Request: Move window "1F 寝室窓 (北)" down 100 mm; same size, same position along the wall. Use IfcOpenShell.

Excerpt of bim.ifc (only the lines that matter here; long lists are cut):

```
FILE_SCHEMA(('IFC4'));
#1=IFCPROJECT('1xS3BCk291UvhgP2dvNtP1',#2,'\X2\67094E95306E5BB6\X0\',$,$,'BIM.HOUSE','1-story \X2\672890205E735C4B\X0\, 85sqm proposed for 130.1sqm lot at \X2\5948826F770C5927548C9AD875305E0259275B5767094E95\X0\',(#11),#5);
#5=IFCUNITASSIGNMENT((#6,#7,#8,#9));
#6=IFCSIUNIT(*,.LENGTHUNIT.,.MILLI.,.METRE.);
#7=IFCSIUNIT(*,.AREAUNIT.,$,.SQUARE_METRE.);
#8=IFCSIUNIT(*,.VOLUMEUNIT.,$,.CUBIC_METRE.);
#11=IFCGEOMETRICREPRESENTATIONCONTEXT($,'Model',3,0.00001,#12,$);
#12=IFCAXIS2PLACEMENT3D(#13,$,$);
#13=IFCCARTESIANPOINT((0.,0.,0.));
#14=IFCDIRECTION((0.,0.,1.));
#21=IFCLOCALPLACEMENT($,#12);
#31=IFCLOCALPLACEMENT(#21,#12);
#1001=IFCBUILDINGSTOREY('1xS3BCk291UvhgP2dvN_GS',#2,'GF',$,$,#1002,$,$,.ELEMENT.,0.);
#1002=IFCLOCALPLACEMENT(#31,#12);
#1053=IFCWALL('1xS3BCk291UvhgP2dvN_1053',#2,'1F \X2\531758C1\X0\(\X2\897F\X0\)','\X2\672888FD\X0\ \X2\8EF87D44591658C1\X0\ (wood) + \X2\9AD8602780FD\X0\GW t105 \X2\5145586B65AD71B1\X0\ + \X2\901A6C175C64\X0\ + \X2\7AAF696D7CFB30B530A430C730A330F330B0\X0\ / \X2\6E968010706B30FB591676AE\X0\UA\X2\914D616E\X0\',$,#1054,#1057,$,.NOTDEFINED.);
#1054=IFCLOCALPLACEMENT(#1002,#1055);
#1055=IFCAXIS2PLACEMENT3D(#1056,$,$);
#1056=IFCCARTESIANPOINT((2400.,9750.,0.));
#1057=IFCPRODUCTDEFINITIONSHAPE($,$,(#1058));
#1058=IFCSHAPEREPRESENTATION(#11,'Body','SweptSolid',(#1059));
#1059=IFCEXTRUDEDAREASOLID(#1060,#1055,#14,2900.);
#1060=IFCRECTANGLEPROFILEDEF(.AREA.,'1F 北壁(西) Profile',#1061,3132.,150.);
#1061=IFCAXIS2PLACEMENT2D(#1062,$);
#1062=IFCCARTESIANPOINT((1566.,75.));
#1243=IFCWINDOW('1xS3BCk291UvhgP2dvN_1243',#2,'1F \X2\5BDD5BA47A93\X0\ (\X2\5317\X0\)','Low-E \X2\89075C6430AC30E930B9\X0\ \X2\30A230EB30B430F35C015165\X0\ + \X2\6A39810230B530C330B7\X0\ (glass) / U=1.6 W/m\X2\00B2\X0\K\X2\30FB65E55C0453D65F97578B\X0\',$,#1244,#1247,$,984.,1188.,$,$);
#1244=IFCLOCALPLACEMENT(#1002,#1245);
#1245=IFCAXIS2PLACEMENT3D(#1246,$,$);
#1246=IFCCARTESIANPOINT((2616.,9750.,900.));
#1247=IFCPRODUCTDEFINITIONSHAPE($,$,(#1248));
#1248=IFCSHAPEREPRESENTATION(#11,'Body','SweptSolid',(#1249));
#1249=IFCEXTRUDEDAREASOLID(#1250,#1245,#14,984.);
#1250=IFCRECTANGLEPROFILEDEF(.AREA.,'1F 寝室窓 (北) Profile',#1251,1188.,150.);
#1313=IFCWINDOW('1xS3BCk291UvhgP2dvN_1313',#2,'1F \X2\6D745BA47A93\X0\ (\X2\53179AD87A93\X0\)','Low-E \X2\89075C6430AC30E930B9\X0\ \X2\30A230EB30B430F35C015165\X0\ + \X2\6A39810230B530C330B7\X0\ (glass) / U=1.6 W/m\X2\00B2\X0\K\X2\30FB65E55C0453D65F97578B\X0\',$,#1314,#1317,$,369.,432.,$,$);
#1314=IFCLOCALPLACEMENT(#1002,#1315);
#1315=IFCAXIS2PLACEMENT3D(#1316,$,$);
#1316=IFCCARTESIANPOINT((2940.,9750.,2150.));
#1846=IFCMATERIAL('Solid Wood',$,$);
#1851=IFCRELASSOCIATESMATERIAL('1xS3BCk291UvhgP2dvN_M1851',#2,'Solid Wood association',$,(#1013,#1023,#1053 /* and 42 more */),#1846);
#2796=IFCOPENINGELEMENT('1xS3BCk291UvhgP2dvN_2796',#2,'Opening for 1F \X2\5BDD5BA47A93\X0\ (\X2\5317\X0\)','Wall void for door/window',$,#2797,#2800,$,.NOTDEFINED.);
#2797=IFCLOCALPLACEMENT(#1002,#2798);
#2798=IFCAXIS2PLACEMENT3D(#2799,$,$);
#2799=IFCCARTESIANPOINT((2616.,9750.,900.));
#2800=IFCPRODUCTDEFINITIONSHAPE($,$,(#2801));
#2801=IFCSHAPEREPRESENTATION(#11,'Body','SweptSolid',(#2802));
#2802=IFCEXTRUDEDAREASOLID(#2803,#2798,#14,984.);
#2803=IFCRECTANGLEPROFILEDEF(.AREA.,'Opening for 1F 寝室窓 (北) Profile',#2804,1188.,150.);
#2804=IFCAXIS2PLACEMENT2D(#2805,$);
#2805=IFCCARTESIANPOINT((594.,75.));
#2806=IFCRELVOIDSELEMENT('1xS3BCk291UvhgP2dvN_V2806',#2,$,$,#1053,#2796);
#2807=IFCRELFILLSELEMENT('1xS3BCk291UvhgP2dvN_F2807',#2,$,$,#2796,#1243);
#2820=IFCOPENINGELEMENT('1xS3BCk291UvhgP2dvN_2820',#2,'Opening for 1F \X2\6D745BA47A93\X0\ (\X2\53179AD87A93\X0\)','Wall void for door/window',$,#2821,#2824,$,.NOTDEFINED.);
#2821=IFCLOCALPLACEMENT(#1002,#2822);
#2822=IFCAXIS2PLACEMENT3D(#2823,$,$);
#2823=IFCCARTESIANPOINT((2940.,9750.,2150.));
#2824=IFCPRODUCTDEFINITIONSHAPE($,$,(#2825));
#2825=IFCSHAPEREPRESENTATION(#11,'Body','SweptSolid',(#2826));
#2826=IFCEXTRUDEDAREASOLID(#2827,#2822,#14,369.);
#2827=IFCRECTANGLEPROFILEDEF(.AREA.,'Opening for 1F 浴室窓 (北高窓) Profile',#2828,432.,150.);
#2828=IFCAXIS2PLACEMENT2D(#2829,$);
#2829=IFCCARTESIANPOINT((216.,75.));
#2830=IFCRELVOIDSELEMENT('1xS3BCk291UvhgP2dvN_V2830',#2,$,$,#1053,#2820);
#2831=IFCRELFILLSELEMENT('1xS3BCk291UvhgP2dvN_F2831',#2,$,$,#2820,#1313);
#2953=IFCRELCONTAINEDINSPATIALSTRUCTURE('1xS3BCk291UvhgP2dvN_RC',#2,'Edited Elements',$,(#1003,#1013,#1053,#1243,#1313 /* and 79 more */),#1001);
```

```python
import numpy as np
import ifcopenshell
import ifcopenshell.api.geometry
import ifcopenshell.util.placement
import ifcopenshell.util.unit

model = ifcopenshell.open("bim.ifc")
unit_scale = ifcopenshell.util.unit.calculate_unit_scale(model)

window = model.by_guid("1xS3BCk291UvhgP2dvN_1243")
opening = window.FillsVoids[0].RelatingOpeningElement
dz = -100.0

shift = np.array([0.0, 0.0, dz])
# The window is not placed relative to its opening, so move both.
for product in (opening, window):
    matrix = ifcopenshell.util.placement.get_local_placement(product.ObjectPlacement)
    matrix[:3, 3] += shift
    ifcopenshell.api.geometry.edit_object_placement(model, product=product, matrix=matrix, is_si=False)

print(f"moved by {dz * unit_scale:+.3f} m")

model.write("bim_rev.ifc")
```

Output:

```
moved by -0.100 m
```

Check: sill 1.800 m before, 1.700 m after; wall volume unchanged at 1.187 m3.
